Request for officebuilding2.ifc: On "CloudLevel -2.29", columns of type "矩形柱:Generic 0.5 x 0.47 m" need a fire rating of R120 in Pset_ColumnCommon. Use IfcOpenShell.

First a look at what the model holds.

```python
import ifcopenshell
import ifcopenshell.util.element

model = ifcopenshell.open("officebuilding2.ifc")
print(model.schema)
storey = next(s for s in model.by_type("IfcBuildingStorey") if s.Name == "CloudLevel -2.29")
columns = [e for e in ifcopenshell.util.element.get_decomposition(storey) if e.is_a("IfcColumn")]
seen = {}
for e in columns:
    element_type = ifcopenshell.util.element.get_type(e)
    key = (element_type.Name if element_type != e and element_type else None, ifcopenshell.util.element.get_pset(e, "Pset_ColumnCommon", "FireRating"))
    seen[key] = seen.get(key, 0) + 1
for (name, value), count in sorted(seen.items(), key=str):
    print(count, "x", name, "|", value)
```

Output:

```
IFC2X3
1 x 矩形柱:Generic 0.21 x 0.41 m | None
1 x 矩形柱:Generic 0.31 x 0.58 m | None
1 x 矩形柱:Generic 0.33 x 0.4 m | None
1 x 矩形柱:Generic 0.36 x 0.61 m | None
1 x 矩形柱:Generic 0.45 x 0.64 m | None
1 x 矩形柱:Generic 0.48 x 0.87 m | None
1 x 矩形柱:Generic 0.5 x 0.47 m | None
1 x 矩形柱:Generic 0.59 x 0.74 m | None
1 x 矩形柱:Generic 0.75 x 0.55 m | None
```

```python
import ifcopenshell
import ifcopenshell.api.pset
import ifcopenshell.util.element

model = ifcopenshell.open("officebuilding2.ifc")

storey = next(s for s in model.by_type("IfcBuildingStorey") if s.Name == "CloudLevel -2.29")
columns = [e for e in ifcopenshell.util.element.get_decomposition(storey) if e.is_a("IfcColumn")]

count = 0
for e in columns:
    element_type = ifcopenshell.util.element.get_type(e)
    if element_type in (None, e) or element_type.Name != "矩形柱:Generic 0.5 x 0.47 m":
        continue
    # add_pset returns the element's existing set when there is one.
    pset = ifcopenshell.api.pset.add_pset(model, product=e, name="Pset_ColumnCommon")
    ifcopenshell.api.pset.edit_pset(model, pset=pset, properties={"FireRating": "R120"})
    count += 1

print(count, "columns updated")

model.write("officebuilding2-out.ifc")
```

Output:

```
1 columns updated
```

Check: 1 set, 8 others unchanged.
